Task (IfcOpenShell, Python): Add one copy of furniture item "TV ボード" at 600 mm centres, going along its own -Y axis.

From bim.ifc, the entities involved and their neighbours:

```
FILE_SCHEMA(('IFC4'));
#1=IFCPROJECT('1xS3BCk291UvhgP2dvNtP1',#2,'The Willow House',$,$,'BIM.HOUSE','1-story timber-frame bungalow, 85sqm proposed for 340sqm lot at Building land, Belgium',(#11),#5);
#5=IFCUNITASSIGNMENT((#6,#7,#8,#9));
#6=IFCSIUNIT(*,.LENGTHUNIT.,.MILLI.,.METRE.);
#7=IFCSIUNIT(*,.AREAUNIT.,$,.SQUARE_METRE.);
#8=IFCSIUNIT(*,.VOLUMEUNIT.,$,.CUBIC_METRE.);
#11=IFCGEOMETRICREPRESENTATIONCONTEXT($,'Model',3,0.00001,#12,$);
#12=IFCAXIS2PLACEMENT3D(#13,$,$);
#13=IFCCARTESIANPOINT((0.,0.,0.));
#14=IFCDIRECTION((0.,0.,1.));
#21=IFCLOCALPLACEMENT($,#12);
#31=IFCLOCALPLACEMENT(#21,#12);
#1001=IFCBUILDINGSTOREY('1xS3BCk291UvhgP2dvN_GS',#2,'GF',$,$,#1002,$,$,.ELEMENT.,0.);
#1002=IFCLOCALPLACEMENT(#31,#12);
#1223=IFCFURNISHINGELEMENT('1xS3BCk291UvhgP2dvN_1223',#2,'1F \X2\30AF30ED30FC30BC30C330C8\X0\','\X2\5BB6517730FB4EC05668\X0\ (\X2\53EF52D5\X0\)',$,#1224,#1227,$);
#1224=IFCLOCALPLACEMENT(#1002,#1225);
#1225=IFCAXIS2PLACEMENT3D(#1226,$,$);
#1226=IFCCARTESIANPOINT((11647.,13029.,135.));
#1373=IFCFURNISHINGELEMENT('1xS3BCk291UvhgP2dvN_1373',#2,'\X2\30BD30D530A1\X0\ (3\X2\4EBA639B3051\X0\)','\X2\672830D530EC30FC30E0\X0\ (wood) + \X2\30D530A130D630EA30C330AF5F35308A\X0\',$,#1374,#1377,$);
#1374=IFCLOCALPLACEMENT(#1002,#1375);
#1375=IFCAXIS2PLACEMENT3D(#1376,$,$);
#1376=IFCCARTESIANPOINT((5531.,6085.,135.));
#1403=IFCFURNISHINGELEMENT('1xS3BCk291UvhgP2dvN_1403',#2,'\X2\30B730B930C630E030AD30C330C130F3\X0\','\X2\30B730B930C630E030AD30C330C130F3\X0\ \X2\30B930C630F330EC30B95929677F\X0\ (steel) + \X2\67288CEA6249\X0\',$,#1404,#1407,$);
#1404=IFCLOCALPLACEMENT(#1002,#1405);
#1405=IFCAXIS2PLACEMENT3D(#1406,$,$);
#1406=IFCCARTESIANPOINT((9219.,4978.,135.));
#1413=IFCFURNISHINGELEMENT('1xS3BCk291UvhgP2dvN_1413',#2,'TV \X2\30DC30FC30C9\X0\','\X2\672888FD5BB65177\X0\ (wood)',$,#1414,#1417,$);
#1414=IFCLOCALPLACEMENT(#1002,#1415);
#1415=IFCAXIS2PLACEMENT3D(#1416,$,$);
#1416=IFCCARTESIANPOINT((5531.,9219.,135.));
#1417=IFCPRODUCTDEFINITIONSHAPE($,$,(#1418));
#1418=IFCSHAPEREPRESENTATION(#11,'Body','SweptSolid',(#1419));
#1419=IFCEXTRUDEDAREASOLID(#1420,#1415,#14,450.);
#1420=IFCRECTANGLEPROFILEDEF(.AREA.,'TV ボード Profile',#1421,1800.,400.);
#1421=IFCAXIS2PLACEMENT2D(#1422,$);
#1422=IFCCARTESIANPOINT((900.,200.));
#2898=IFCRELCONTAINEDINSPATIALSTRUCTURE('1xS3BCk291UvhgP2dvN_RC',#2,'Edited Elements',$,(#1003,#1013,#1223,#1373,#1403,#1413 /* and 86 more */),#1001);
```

```python
import ifcopenshell
import ifcopenshell.api.geometry
import ifcopenshell.api.root
import ifcopenshell.util.element
import ifcopenshell.util.placement
import ifcopenshell.util.unit

model = ifcopenshell.open("bim.ifc")
unit_scale = ifcopenshell.util.unit.calculate_unit_scale(model)


def reuse_history(source, copy):
    """copy_class also copies each property set's owner history, people and application; keep the originals."""
    for rel in copy.IsDefinedBy:
        if rel.is_a("IfcRelDefinesByProperties") and (history := rel.RelatingPropertyDefinition.OwnerHistory):
            rel.RelatingPropertyDefinition.OwnerHistory = source.OwnerHistory
            ifcopenshell.util.element.remove_deep2(model, history)


source = model.by_guid("1xS3BCk291UvhgP2dvN_1413")
base = ifcopenshell.util.placement.get_local_placement(source.ObjectPlacement)
step = -base[:3, 1] * 0.6 / unit_scale

for i in range(1, 2):
    copy = ifcopenshell.api.root.copy_class(model, product=source)
    copy.Representation = ifcopenshell.util.element.copy_deep(
        model, source.Representation, exclude=["IfcGeometricRepresentationContext", "IfcRepresentationMap"]
    )
    reuse_history(source, copy)
    matrix = base.copy()
    matrix[:3, 3] += i * step
    print("added at", matrix[:3, 3].round(3) + 0.0)
    ifcopenshell.api.geometry.edit_object_placement(model, product=copy, matrix=matrix, is_si=False)

model.write("bim_rev.ifc")
```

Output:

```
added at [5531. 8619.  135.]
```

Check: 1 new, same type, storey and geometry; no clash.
